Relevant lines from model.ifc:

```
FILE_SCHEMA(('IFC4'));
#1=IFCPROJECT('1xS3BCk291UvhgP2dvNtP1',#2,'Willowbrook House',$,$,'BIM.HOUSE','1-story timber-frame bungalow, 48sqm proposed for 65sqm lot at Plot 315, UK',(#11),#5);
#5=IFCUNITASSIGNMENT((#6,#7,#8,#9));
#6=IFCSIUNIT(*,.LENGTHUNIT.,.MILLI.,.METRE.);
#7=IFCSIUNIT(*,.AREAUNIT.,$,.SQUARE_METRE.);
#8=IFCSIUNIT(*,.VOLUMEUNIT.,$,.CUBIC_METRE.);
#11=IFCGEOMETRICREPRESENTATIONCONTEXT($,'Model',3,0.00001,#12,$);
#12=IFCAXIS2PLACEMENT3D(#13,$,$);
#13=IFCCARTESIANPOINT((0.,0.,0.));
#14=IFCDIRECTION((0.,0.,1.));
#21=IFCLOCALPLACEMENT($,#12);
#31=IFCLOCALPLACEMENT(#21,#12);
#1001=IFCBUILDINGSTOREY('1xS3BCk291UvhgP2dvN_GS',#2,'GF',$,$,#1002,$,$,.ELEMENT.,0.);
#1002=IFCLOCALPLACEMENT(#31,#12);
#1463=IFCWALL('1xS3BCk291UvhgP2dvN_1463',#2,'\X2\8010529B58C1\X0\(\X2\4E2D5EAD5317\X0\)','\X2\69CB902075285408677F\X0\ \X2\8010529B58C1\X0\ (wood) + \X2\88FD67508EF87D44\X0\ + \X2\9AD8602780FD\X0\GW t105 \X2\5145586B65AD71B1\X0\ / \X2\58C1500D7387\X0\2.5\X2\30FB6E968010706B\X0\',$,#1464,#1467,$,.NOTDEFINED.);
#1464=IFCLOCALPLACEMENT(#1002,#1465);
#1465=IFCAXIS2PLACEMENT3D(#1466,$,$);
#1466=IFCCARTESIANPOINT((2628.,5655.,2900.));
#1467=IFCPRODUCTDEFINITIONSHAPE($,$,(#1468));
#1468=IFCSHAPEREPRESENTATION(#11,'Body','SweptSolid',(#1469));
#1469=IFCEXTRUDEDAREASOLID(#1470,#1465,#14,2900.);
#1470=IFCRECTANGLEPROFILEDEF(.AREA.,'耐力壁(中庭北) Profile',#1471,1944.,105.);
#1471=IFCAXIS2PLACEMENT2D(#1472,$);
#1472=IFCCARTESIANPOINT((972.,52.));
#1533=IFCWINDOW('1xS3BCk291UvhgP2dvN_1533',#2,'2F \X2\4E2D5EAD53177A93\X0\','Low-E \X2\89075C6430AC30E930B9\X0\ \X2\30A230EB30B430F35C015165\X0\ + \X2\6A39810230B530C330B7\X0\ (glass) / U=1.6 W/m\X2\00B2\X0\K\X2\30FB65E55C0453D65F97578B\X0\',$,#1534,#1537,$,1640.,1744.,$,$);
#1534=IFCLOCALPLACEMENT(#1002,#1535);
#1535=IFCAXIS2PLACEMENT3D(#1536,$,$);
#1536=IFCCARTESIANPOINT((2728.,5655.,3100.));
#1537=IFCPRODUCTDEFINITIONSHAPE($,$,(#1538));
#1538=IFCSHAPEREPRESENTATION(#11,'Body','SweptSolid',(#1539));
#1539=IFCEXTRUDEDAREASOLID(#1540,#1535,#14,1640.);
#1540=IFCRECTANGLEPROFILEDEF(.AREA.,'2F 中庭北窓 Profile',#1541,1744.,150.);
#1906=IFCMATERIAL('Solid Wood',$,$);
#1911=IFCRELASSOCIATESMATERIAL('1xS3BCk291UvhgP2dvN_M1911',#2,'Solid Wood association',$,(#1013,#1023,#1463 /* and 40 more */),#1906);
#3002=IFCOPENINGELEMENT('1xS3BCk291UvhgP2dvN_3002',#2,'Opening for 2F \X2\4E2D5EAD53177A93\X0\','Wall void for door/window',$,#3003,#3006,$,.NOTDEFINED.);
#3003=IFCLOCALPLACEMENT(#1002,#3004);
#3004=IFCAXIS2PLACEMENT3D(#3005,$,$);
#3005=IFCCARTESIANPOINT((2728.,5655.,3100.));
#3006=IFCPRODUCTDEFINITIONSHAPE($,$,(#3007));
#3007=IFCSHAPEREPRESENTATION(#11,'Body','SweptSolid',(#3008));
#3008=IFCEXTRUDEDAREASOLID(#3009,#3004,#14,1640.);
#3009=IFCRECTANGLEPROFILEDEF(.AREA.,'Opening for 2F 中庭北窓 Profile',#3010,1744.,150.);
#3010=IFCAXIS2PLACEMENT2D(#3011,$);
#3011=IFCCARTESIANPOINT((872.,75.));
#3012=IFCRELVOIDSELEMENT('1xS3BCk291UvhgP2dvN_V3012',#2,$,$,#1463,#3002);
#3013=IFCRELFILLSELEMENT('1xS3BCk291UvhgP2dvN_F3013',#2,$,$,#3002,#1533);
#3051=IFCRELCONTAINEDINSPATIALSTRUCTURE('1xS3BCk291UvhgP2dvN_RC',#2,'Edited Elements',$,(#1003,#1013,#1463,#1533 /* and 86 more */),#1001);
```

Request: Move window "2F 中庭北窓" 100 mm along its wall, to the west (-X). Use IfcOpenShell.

```python
import ifcopenshell
import ifcopenshell.api.geometry
import ifcopenshell.util.placement

model = ifcopenshell.open("model.ifc")

window = model.by_id(1533)
opening = window.FillsVoids[0].RelatingOpeningElement
wall = opening.VoidsElements[0].RelatingBuildingElement

wall_matrix = ifcopenshell.util.placement.get_local_placement(wall.ObjectPlacement)
shift = wall_matrix[:3, 0] * -100.0
before = ifcopenshell.util.placement.get_local_placement(window.ObjectPlacement)[:3, 3].copy()

# The window is not placed relative to its opening, so move both.
for product in (opening, window):
    matrix = ifcopenshell.util.placement.get_local_placement(product.ObjectPlacement)
    matrix[:3, 3] += shift
    ifcopenshell.api.geometry.edit_object_placement(model, product=product, matrix=matrix, is_si=False)

after = ifcopenshell.util.placement.get_local_placement(window.ObjectPlacement)[:3, 3]
print("window moved by", (after - before).round(3) + 0.0)

model.write("model-out.ifc")
```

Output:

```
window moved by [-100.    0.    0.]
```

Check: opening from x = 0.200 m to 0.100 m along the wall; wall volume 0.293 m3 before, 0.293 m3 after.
